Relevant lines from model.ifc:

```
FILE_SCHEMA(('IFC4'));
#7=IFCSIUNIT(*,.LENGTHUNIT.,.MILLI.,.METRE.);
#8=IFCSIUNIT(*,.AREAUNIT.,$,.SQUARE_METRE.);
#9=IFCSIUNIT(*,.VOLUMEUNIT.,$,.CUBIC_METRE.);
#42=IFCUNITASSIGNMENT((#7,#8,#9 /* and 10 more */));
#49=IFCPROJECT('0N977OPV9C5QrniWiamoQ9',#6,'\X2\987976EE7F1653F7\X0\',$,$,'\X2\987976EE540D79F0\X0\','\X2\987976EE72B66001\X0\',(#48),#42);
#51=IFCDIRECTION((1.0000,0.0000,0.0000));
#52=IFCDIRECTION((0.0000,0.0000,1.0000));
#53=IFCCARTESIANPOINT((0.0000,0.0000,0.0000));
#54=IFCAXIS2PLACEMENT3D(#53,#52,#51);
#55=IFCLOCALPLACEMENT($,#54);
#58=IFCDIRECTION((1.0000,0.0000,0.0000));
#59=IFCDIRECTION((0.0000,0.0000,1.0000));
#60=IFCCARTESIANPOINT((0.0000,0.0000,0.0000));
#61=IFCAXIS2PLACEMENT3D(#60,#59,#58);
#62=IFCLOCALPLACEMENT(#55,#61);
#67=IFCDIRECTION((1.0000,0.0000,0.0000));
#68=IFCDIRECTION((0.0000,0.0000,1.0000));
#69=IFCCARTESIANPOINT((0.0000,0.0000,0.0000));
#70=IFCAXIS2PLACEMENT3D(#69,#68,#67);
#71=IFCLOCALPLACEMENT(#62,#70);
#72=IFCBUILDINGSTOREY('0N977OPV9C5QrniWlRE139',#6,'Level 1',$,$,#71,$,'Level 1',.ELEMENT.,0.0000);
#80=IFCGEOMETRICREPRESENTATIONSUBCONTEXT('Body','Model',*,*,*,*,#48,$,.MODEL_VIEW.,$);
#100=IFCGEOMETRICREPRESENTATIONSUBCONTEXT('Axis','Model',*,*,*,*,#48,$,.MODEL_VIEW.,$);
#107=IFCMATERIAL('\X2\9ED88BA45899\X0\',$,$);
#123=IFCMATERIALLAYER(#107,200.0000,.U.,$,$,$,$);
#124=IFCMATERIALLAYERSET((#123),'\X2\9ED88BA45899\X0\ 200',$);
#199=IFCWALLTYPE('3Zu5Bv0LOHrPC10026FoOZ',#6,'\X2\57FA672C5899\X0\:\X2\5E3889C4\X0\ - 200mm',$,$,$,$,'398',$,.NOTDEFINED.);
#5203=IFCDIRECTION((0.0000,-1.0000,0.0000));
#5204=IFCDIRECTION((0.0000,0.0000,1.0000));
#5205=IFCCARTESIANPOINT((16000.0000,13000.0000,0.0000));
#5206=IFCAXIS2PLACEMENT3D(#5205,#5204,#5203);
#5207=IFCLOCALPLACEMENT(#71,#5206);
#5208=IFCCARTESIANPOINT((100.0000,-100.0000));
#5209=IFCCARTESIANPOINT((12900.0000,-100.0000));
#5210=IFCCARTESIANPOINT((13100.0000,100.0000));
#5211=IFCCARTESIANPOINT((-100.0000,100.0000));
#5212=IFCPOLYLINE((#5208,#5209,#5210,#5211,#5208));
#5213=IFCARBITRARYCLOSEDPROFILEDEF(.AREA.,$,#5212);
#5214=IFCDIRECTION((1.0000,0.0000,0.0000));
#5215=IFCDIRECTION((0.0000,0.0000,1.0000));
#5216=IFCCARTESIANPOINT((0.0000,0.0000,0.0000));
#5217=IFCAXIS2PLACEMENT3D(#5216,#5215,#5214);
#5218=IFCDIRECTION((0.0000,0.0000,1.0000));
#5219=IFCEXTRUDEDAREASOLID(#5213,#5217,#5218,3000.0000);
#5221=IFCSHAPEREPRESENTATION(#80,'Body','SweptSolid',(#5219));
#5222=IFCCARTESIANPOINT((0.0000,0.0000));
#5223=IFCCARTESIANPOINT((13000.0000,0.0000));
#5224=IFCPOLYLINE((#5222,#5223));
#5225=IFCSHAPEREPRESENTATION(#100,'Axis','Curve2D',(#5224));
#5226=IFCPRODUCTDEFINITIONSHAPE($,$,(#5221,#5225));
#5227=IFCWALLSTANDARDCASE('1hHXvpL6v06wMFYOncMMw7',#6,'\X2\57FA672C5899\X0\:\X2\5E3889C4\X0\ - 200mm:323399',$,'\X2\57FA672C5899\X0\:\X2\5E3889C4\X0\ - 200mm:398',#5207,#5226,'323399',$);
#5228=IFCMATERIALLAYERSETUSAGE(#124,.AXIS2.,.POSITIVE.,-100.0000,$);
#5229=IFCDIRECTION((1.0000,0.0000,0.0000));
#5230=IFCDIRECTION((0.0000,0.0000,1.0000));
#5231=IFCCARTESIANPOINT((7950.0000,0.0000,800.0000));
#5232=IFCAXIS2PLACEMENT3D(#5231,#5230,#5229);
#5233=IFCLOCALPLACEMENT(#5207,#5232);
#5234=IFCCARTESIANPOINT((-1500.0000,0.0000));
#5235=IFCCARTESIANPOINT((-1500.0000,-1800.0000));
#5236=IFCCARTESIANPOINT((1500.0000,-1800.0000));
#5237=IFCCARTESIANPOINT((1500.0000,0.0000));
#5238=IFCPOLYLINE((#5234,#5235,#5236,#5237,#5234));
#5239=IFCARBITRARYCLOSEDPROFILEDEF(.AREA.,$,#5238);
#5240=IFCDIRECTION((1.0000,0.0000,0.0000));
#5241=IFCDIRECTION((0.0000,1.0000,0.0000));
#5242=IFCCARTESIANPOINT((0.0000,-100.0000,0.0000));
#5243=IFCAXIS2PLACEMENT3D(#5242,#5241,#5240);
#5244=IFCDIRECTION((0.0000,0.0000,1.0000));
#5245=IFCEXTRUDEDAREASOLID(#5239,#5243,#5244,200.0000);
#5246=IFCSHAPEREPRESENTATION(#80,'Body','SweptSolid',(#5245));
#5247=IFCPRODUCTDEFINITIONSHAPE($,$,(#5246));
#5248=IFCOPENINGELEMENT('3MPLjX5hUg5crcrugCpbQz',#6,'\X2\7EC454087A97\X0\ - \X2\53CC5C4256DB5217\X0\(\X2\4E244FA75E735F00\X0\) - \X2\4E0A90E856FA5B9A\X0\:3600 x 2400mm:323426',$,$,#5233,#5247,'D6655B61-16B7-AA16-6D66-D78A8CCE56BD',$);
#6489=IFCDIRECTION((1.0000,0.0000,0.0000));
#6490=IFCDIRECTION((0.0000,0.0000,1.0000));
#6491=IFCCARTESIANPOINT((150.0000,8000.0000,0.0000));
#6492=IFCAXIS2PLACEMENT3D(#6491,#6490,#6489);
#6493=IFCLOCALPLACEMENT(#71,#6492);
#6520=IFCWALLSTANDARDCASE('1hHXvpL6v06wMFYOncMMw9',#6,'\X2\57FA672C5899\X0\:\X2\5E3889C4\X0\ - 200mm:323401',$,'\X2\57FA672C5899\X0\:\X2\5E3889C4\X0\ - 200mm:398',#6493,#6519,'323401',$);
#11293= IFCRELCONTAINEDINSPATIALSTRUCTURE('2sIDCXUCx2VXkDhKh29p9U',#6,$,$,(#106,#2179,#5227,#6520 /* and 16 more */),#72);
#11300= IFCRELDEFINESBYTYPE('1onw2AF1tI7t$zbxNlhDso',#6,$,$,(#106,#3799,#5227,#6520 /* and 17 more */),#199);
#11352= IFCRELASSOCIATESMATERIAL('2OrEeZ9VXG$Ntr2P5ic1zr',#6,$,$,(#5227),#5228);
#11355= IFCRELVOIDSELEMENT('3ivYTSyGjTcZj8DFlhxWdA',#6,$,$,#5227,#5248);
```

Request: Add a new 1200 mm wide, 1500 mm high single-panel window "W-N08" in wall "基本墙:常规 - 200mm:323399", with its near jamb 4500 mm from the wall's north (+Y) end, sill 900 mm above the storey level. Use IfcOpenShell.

```python
import numpy as np
import ifcopenshell
import ifcopenshell.api.feature
import ifcopenshell.api.geometry
import ifcopenshell.api.root
import ifcopenshell.api.spatial
import ifcopenshell.geom
import ifcopenshell.util.element
import ifcopenshell.util.placement
import ifcopenshell.util.representation
import ifcopenshell.util.shape
import ifcopenshell.util.unit

model = ifcopenshell.open("model.ifc")
unit_scale = ifcopenshell.util.unit.calculate_unit_scale(model)
settings = ifcopenshell.geom.settings()


def volume(element):
    """Net volume in cubic metres, openings subtracted."""
    shape = ifcopenshell.geom.create_shape(settings, element)
    return ifcopenshell.util.shape.get_volume(shape.geometry)


wall = model.by_guid("1hHXvpL6v06wMFYOncMMw7")
storey = ifcopenshell.util.element.get_container(wall, ifc_class="IfcBuildingStorey")
context = ifcopenshell.util.representation.get_context(model, "Model", "Body", "MODEL_VIEW")
before = volume(wall)

width, height, from_end, sill = 1.2, 1.5, 4.5, 0.9  # metres

# The wall runs along its own X axis, and the end named is its -X end.
wall_shape = ifcopenshell.geom.create_shape(settings, wall)
x, y, z = ifcopenshell.util.shape.get_vertices(wall_shape.geometry).T
start = x.min() + from_end
face, thickness = float(y.min()), float(y.max() - y.min())
wall_matrix = ifcopenshell.util.placement.get_local_placement(wall.ObjectPlacement)
level = ifcopenshell.util.placement.get_local_placement(storey.ObjectPlacement)[2, 3]


def in_wall(x, y):
    """Placement at x, y metres in the wall's axes, at sill height."""
    matrix = wall_matrix.copy()
    matrix[:, 3] = wall_matrix @ np.array([x / unit_scale, y / unit_scale, 0.0, 1.0])
    matrix[2, 3] = level + sill / unit_scale
    return matrix


# Opening: a box that overshoots both wall faces by 50 mm.
opening = ifcopenshell.api.root.create_entity(model, ifc_class="IfcOpeningElement", predefined_type="OPENING")
box = ifcopenshell.api.geometry.add_wall_representation(
    model, context=context, length=width, height=height, thickness=thickness + 0.1
)
ifcopenshell.api.geometry.assign_representation(model, product=opening, representation=box)
ifcopenshell.api.geometry.edit_object_placement(model, product=opening, matrix=in_wall(start, face - 0.05), is_si=False)
ifcopenshell.api.feature.add_feature(model, feature=opening, element=wall)

window = ifcopenshell.api.root.create_entity(model, ifc_class="IfcWindow", name="W-N08", predefined_type="WINDOW")
window.OverallWidth, window.OverallHeight = width / unit_scale, height / unit_scale
window.PartitioningType = "SINGLE_PANEL"
body = ifcopenshell.api.geometry.add_window_representation(
    model,
    context=context,
    overall_width=window.OverallWidth,
    overall_height=window.OverallHeight,
    partition_type="SINGLE_PANEL",
)
ifcopenshell.api.geometry.assign_representation(model, product=window, representation=body)
ifcopenshell.api.spatial.assign_container(model, products=[window], relating_structure=storey)
ifcopenshell.api.feature.add_filling(model, opening=opening, element=window)

# Centre the window in the wall's thickness.
ifcopenshell.api.geometry.edit_object_placement(model, product=window, matrix=in_wall(start, face), is_si=False)
window_shape = ifcopenshell.geom.create_shape(settings, window)
depth = ifcopenshell.util.shape.get_vertices(window_shape.geometry)[:, 1]
offset = face + thickness / 2 - (depth.min() + depth.max()) / 2
ifcopenshell.api.geometry.edit_object_placement(model, product=window, matrix=in_wall(start, offset), is_si=False)

after = volume(wall)

print(f"wall volume {before:.3f} -> {after:.3f} m3")

model.write("model_edited.ifc")
```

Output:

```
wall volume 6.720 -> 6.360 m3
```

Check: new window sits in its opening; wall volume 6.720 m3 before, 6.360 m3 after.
